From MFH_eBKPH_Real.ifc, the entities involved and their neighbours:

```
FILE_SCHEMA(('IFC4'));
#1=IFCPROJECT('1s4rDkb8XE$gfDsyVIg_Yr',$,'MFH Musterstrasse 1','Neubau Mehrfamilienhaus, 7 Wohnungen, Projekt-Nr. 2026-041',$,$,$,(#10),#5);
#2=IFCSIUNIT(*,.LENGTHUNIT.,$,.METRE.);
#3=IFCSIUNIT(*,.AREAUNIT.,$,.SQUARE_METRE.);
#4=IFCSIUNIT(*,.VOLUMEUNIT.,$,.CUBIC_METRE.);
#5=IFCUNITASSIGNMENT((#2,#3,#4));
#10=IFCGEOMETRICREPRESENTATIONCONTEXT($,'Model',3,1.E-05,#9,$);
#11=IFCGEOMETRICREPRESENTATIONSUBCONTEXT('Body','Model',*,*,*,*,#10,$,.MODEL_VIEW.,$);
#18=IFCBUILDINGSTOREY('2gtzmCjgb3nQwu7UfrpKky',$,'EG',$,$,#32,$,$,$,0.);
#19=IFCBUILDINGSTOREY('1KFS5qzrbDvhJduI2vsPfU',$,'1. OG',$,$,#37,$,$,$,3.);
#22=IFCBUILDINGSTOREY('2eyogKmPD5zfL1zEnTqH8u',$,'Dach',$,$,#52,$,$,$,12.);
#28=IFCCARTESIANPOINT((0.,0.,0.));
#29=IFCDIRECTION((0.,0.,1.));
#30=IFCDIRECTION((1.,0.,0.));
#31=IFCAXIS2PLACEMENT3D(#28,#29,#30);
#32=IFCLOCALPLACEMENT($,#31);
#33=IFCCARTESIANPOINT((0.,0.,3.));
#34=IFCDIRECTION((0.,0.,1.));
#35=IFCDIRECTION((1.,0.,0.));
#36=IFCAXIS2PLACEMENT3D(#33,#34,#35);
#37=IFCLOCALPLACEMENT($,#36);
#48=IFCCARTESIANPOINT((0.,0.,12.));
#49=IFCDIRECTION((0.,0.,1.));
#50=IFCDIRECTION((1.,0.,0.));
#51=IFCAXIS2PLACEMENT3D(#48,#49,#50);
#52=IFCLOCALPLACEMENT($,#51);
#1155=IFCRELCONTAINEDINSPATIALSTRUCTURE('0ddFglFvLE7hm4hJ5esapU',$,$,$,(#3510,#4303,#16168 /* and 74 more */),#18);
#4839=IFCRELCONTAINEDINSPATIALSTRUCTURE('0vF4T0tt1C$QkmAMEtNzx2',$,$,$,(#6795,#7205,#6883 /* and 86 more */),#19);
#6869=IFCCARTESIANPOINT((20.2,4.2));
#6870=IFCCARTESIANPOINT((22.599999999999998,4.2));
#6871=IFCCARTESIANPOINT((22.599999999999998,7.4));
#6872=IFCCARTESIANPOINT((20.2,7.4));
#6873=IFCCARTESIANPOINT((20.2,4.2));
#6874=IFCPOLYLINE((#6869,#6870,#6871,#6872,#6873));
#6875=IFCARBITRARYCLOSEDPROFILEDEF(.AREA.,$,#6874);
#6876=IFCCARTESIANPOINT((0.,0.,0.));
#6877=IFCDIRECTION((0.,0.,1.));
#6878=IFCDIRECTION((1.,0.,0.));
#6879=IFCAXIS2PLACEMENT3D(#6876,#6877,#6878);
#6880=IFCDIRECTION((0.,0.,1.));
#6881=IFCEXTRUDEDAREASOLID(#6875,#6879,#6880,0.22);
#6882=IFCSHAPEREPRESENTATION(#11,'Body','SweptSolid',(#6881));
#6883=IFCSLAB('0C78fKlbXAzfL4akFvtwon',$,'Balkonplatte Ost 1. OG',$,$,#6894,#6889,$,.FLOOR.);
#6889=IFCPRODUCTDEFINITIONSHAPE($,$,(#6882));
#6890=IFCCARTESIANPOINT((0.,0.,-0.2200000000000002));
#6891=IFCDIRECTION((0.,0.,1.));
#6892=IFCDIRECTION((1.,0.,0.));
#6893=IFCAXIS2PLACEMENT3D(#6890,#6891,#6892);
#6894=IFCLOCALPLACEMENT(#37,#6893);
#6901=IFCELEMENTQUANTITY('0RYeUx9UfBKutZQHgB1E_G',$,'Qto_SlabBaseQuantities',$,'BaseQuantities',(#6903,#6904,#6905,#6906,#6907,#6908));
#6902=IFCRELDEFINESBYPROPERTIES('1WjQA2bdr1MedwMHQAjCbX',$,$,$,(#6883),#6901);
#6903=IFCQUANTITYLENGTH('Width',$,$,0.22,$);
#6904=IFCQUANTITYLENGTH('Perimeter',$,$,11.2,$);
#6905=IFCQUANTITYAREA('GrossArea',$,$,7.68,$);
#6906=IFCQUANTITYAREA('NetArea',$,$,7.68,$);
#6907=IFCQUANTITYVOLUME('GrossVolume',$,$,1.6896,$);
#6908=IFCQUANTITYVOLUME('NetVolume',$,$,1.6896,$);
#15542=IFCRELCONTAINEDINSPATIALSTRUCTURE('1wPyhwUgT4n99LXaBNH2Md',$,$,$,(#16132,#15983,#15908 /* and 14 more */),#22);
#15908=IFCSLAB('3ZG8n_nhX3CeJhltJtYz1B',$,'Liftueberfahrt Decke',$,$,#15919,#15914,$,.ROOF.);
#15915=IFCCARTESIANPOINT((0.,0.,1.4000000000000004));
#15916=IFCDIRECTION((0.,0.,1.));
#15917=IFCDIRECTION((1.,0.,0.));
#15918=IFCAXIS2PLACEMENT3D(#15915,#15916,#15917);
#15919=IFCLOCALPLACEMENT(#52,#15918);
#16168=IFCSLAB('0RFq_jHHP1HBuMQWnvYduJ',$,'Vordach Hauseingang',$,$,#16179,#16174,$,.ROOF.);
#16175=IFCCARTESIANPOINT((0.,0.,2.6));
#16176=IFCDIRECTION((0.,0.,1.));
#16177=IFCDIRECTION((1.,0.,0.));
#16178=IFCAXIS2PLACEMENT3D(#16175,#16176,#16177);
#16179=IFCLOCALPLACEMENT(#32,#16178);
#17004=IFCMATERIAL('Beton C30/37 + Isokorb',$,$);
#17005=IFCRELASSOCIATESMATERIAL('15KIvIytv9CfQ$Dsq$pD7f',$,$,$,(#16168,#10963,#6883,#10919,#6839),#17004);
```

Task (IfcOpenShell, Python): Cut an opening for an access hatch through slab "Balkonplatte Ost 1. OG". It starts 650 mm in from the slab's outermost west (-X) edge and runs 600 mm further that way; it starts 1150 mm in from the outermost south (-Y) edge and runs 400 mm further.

```python
import numpy as np
import ifcopenshell
import ifcopenshell.api.feature
import ifcopenshell.api.geometry
import ifcopenshell.api.pset
import ifcopenshell.api.root
import ifcopenshell.geom
import ifcopenshell.util.element
import ifcopenshell.util.placement
import ifcopenshell.util.representation
import ifcopenshell.util.shape
import ifcopenshell.util.unit

model = ifcopenshell.open("MFH_eBKPH_Real.ifc")
unit_scale = ifcopenshell.util.unit.calculate_unit_scale(model)
area_scale = ifcopenshell.util.unit.calculate_unit_scale(model, "AREAUNIT")
volume_scale = ifcopenshell.util.unit.calculate_unit_scale(model, "VOLUMEUNIT")
settings = ifcopenshell.geom.settings()


def volume(element):
    """Net volume in cubic metres, openings subtracted."""
    shape = ifcopenshell.geom.create_shape(settings, element)
    return ifcopenshell.util.shape.get_volume(shape.geometry)


slab = model.by_id(6883)
before = volume(slab)

# Extent in the slab's own axes, in metres. The edges named are its -X and -Y sides.
slab_shape = ifcopenshell.geom.create_shape(settings, slab)
vertices = ifcopenshell.util.shape.get_vertices(slab_shape.geometry)
x_min, y_min, bottom = vertices.min(axis=0)
top = vertices[:, 2].max()

opening = ifcopenshell.api.root.create_entity(model, ifc_class="IfcOpeningElement", name="Access hatch opening", predefined_type="OPENING")
context = ifcopenshell.util.representation.get_context(model, "Model", "Body", "MODEL_VIEW")
width, depth = 0.6, 0.4
outline = [(0.0, 0.0), (width, 0.0), (width, depth), (0.0, depth), (0.0, 0.0)]
# Overshoot both faces by 50 mm so the cut is clean.
shape = ifcopenshell.api.geometry.add_slab_representation(
    model, context=context, depth=top - bottom + 0.1, polyline=outline
)
ifcopenshell.api.geometry.assign_representation(model, product=opening, representation=shape)

matrix = ifcopenshell.util.placement.get_local_placement(slab.ObjectPlacement)
matrix[:, 3] = matrix @ np.append(np.array([x_min + 0.65, y_min + 1.15, bottom - 0.05]) / unit_scale, 1.0)
ifcopenshell.api.geometry.edit_object_placement(model, product=opening, matrix=matrix, is_si=False)
ifcopenshell.api.feature.add_feature(model, feature=opening, element=slab)

after = volume(slab)

# Update the slab's stored quantities.
qto = model.by_id(ifcopenshell.util.element.get_pset(slab, "Qto_SlabBaseQuantities", should_inherit=False)["id"])
ifcopenshell.api.pset.edit_qto(model, qto=qto, properties={
    "NetArea": after / (top - bottom) / area_scale,
    "NetVolume": after / volume_scale,
})

print(f"slab volume {before:.3f} -> {after:.3f} m3")

model.write("MFH_eBKPH_Real_updated.ifc")
```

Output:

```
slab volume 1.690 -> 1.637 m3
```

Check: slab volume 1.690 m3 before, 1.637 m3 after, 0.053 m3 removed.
